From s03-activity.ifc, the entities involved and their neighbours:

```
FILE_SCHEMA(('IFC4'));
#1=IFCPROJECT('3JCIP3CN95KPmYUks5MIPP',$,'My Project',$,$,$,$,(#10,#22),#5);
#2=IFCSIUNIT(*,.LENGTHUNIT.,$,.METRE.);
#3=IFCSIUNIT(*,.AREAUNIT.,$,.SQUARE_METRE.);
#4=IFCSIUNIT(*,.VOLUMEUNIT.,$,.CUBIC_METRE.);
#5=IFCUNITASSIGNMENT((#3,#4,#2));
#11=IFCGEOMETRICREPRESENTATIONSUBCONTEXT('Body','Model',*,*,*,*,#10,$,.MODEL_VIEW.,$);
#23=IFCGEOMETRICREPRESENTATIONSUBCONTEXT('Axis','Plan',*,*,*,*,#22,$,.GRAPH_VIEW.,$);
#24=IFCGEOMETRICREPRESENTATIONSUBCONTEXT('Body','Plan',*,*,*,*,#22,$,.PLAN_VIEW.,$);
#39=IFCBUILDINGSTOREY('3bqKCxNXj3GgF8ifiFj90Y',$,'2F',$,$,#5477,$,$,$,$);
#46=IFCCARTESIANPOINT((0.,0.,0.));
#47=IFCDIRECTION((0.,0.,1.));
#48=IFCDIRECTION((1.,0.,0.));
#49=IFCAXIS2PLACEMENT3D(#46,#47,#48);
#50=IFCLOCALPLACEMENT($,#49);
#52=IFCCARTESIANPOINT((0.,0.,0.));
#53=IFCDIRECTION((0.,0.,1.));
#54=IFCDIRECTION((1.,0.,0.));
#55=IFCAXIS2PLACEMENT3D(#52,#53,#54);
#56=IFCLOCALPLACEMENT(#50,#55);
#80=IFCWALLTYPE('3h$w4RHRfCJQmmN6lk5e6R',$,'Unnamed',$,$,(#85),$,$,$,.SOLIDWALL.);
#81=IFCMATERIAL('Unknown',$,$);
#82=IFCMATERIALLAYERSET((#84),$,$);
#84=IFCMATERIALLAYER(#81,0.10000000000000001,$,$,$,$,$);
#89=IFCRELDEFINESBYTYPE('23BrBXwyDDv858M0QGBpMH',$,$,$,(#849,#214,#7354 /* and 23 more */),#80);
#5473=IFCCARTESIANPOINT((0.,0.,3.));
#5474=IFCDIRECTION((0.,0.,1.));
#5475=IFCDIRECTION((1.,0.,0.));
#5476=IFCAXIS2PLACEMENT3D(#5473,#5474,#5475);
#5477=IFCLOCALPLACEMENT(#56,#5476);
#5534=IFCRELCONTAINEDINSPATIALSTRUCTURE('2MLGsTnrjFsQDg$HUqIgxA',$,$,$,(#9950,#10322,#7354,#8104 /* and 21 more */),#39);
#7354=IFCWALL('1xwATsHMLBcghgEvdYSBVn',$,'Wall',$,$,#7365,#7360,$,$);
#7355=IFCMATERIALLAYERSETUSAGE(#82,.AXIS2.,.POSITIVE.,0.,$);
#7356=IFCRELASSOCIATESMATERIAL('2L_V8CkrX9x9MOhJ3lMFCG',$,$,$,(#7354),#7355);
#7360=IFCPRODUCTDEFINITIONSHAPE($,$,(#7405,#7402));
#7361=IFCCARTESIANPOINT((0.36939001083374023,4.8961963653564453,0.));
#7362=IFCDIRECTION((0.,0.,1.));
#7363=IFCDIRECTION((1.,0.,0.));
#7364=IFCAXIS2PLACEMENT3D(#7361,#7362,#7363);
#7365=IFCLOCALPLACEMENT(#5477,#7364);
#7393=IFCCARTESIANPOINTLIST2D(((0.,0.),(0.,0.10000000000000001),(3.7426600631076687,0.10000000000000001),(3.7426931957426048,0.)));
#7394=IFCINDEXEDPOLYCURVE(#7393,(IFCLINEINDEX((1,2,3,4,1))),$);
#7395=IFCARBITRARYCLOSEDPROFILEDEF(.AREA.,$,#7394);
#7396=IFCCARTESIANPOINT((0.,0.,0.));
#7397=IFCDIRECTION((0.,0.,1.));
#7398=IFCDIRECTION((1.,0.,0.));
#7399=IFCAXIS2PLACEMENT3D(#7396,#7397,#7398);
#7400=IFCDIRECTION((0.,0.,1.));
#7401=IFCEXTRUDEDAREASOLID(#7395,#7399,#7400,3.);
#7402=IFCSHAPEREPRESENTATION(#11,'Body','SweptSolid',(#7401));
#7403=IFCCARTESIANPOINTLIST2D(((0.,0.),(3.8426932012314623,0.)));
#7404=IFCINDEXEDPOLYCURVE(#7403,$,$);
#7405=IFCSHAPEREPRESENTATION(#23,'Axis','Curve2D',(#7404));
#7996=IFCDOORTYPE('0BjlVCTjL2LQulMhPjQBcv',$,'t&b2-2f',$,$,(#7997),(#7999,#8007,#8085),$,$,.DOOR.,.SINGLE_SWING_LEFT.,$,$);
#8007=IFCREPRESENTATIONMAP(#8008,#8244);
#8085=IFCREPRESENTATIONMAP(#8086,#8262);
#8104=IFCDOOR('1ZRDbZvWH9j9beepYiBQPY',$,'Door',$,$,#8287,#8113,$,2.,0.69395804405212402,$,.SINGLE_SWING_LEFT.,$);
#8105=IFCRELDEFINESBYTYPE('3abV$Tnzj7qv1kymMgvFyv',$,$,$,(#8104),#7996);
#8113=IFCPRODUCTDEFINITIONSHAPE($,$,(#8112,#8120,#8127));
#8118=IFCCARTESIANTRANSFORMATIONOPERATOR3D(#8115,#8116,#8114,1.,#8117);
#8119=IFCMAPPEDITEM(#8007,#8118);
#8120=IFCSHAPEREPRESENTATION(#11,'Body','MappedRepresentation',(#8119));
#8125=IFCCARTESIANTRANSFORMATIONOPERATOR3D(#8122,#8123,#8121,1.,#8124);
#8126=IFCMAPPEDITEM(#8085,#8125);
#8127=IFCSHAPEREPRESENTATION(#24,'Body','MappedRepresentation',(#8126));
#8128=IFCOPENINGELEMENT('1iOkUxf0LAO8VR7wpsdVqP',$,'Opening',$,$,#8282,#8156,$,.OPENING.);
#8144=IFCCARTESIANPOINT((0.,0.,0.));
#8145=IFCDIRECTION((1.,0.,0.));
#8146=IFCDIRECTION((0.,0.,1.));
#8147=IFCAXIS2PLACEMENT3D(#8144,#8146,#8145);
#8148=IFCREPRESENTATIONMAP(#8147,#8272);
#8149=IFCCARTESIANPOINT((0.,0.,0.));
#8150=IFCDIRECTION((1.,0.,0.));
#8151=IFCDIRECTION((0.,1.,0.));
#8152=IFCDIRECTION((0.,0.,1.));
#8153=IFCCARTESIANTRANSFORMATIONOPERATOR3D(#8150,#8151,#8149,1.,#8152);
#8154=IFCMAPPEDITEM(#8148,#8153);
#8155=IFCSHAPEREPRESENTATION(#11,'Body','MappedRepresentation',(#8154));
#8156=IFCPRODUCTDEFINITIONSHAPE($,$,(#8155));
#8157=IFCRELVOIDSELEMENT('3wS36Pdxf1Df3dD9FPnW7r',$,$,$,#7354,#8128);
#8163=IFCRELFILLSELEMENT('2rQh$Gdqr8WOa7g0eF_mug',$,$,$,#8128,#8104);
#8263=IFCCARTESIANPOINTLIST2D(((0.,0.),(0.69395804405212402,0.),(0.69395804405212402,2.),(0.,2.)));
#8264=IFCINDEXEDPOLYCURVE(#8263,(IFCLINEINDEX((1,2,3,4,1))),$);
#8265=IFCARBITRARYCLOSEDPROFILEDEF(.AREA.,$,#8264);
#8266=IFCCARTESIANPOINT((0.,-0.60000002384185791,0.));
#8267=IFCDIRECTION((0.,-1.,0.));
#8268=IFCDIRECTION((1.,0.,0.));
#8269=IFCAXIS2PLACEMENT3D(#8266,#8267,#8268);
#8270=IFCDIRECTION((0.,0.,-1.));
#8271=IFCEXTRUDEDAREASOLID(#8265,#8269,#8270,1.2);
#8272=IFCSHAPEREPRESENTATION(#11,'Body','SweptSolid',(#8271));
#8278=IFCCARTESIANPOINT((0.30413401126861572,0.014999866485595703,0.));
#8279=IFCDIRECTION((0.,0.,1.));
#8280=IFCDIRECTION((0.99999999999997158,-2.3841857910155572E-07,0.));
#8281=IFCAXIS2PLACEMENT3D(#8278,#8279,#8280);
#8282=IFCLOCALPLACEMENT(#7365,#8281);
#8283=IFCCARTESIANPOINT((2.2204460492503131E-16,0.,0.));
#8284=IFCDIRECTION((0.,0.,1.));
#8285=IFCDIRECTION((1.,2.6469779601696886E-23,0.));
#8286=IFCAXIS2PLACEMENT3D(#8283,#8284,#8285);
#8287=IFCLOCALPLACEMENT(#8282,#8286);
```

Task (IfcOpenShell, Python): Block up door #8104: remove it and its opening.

```python
import ifcopenshell
import ifcopenshell.api.feature
import ifcopenshell.api.root
import ifcopenshell.geom
import ifcopenshell.util.shape

model = ifcopenshell.open("s03-activity.ifc")
settings = ifcopenshell.geom.settings()


def volume(element):
    """Net volume in cubic metres, openings subtracted."""
    shape = ifcopenshell.geom.create_shape(settings, element)
    return ifcopenshell.util.shape.get_volume(shape.geometry)


door = model.by_guid("1ZRDbZvWH9j9beepYiBQPY")
opening = door.FillsVoids[0].RelatingOpeningElement
wall = opening.VoidsElements[0].RelatingBuildingElement
before = volume(wall)

ifcopenshell.api.root.remove_product(model, product=door)
ifcopenshell.api.feature.remove_feature(model, feature=opening)

after = volume(wall)

print(f"wall volume {before:.3f} -> {after:.3f} m3")

model.write("s03-activity-out.ifc")
```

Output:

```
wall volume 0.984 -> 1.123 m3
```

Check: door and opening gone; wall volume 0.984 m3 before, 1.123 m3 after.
